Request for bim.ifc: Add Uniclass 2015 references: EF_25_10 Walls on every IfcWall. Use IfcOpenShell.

First a look at what the model holds.

```python
import ifcopenshell

model = ifcopenshell.open("bim.ifc")
print(model.schema)
print("classifications:", [c.Name for c in model.by_type("IfcClassification")])
for ifc_class in ("IfcDoor", "IfcRoof", "IfcStair", "IfcWall", "IfcWindow"):
    print(ifc_class, len(model.by_type(ifc_class)))
```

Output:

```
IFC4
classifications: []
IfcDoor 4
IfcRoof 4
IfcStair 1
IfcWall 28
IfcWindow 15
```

```python
import ifcopenshell
import ifcopenshell.api.classification

model = ifcopenshell.open("bim.ifc")

system = ifcopenshell.api.classification.add_classification(model, classification="Uniclass 2015")

codes = {
    "IfcWall": ("EF_25_10", "Walls"),
}
for ifc_class, (code, name) in codes.items():
    products = model.by_type(ifc_class)
    ifcopenshell.api.classification.add_reference(
        model, products=products, classification=system, identification=code, name=name
    )
    print(code, len(products))

model.write("bim_edited.ifc")
```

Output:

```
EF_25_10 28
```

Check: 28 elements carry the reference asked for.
